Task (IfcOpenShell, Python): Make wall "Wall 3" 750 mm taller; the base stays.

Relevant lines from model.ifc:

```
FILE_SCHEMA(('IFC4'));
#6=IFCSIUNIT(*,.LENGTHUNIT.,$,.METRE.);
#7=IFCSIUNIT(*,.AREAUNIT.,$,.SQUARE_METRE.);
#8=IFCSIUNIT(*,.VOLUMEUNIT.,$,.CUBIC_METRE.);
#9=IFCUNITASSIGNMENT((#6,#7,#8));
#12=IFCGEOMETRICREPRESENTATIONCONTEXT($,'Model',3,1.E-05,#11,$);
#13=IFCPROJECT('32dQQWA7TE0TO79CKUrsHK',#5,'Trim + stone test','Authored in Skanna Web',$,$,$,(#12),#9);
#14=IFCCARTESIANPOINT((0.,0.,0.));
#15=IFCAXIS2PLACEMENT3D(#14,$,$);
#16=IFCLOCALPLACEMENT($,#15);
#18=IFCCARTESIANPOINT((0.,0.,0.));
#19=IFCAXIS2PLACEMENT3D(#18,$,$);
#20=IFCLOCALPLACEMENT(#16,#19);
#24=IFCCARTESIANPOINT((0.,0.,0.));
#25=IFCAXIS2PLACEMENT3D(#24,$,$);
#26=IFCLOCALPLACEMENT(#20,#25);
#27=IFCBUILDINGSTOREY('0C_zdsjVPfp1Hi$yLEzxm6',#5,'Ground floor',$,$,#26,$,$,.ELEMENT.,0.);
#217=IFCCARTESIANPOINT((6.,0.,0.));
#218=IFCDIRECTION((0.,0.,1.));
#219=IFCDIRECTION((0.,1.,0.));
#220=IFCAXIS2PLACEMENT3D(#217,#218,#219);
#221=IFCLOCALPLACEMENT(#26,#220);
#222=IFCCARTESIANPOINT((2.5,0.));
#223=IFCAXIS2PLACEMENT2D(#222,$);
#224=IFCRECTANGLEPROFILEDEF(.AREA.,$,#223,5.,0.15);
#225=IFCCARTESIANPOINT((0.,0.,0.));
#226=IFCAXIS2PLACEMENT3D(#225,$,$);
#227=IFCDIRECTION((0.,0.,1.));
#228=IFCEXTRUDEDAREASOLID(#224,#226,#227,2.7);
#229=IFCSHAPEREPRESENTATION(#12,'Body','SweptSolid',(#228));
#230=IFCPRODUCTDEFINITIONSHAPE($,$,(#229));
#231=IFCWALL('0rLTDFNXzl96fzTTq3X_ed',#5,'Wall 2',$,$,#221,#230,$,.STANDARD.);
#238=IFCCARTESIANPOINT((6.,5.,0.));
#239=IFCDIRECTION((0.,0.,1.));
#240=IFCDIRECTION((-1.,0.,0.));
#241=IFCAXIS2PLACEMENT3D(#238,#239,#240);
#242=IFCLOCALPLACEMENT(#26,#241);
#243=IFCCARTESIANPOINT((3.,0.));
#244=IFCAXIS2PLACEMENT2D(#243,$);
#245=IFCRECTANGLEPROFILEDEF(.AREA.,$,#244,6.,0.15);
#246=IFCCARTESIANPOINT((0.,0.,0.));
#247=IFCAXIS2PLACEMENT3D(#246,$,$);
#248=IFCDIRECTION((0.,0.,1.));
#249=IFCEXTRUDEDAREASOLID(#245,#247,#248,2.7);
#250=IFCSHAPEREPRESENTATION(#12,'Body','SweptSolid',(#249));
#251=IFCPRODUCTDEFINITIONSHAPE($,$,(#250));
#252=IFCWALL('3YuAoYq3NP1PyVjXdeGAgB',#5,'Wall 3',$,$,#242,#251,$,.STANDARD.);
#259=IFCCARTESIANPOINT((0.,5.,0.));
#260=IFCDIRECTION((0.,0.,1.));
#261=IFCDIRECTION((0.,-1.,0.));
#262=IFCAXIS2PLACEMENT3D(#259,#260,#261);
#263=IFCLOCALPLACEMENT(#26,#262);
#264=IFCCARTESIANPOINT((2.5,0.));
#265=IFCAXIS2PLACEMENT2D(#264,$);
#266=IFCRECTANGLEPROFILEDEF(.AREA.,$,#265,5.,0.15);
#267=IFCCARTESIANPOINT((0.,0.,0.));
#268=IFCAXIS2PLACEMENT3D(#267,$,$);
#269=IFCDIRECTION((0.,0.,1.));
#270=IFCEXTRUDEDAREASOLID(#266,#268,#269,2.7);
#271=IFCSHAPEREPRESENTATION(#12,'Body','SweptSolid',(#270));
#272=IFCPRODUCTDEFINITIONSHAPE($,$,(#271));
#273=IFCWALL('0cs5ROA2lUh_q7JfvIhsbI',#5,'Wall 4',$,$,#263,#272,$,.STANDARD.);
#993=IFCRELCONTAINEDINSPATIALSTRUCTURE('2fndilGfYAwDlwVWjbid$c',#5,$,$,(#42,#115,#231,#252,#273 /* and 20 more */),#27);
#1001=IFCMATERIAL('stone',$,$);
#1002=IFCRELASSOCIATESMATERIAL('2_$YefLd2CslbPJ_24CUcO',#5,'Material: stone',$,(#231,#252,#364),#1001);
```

```python
import ifcopenshell
import ifcopenshell.geom
import ifcopenshell.util.shape

model = ifcopenshell.open("model.ifc")
settings = ifcopenshell.geom.settings()


def volume(element):
    """Net volume in cubic metres, openings subtracted."""
    shape = ifcopenshell.geom.create_shape(settings, element)
    return ifcopenshell.util.shape.get_volume(shape.geometry)


wall = model.by_guid("3YuAoYq3NP1PyVjXdeGAgB")
before = volume(wall)

body = next(r for r in wall.Representation.Representations if r.RepresentationIdentifier == "Body")
solid = body.Items[0]
old_height = solid.Depth
solid.Depth += 0.75
after = volume(wall)

print(f"height {old_height:g} -> {solid.Depth:g}, volume {before:.3f} -> {after:.3f} m3")

model.write("model_v2.ifc")
```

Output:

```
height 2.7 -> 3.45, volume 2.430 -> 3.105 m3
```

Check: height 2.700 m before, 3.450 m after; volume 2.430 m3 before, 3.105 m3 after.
